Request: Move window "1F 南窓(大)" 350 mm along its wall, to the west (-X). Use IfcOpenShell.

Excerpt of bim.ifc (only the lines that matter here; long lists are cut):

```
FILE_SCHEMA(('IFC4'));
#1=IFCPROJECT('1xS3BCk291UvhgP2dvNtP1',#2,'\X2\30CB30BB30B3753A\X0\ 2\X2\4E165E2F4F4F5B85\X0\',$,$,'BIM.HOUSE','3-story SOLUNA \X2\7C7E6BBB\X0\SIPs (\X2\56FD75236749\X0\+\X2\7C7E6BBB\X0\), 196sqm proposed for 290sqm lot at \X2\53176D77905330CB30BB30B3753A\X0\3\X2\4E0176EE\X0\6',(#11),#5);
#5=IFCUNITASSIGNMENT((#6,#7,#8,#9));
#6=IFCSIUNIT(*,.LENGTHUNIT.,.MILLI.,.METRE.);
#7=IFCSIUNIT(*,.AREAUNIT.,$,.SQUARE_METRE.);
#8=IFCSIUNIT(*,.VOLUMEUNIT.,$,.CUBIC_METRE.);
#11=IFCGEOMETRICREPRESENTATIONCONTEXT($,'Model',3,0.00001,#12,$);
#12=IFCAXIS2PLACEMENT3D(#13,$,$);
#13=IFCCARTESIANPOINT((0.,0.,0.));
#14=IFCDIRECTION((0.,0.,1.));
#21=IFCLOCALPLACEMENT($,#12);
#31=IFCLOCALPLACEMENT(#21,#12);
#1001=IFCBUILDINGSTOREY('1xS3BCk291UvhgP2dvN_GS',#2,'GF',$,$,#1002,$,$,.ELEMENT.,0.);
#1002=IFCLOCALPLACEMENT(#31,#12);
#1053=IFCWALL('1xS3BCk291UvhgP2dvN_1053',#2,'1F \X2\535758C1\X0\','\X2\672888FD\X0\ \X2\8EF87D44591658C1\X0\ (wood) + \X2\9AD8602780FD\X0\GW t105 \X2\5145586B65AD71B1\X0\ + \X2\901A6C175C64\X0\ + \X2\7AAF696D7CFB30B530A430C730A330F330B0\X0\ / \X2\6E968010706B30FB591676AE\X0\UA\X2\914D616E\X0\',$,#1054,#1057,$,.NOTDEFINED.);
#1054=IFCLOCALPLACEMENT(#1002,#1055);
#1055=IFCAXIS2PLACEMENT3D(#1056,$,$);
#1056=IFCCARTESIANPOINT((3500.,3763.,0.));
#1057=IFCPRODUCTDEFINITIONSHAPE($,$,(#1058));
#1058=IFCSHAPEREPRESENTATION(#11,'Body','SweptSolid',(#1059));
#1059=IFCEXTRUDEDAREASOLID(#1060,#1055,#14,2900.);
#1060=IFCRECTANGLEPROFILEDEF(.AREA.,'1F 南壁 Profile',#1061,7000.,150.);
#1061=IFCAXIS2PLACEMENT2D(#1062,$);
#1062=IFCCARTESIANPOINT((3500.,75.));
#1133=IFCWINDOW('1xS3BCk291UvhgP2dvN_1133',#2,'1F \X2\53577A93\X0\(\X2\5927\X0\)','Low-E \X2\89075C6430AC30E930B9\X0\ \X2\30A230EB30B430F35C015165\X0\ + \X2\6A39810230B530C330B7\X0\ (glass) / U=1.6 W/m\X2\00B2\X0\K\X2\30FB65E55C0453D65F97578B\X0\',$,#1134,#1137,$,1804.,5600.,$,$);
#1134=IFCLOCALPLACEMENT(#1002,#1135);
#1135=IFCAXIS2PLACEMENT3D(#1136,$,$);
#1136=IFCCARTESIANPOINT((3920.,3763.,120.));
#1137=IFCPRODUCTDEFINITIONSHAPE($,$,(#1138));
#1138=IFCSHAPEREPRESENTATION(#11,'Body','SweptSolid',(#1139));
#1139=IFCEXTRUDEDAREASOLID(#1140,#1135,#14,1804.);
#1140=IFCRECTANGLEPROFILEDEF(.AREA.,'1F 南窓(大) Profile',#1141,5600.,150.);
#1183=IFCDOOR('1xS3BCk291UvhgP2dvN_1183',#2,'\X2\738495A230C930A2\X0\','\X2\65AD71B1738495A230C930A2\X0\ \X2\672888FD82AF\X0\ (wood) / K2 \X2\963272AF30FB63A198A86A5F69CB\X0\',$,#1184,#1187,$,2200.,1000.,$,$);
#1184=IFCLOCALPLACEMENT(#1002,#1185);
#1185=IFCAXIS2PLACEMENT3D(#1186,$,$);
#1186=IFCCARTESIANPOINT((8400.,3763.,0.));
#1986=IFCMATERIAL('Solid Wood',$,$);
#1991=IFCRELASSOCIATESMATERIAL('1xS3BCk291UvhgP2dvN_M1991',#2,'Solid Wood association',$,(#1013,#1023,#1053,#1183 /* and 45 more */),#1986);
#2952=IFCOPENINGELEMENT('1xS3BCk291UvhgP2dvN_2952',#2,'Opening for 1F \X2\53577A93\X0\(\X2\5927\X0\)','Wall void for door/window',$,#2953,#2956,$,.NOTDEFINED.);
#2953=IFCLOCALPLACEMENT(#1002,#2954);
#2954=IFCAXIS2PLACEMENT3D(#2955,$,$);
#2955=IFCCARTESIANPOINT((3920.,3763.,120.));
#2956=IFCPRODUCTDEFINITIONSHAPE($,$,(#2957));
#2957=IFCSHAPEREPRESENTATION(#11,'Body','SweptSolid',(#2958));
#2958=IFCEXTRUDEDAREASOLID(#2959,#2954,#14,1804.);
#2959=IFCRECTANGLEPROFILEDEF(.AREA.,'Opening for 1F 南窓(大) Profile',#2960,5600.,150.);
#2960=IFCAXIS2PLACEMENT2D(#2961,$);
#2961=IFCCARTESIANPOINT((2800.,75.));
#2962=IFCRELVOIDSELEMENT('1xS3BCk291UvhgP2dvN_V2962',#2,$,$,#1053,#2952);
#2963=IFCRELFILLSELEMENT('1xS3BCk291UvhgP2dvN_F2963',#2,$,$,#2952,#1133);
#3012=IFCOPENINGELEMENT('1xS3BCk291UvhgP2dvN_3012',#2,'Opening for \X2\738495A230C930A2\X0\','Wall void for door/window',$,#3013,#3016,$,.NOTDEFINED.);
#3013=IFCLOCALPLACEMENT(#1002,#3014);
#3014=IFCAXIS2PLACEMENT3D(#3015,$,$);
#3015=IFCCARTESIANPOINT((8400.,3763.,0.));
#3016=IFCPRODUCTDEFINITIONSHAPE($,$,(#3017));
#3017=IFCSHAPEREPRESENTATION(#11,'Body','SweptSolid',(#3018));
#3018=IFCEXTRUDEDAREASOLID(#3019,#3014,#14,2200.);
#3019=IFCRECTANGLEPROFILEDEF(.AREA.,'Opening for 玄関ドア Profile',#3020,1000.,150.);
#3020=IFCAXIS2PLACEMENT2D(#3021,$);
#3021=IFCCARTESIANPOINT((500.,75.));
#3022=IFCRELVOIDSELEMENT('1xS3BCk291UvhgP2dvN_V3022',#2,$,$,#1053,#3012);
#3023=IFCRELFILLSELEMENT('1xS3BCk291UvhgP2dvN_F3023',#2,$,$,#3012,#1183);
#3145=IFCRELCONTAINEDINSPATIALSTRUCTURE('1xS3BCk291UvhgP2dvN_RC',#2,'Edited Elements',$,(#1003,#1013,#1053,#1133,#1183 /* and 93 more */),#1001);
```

```python
import ifcopenshell
import ifcopenshell.api.geometry
import ifcopenshell.util.placement

model = ifcopenshell.open("bim.ifc")

window = model.by_id(1133)
opening = window.FillsVoids[0].RelatingOpeningElement
wall = opening.VoidsElements[0].RelatingBuildingElement

wall_matrix = ifcopenshell.util.placement.get_local_placement(wall.ObjectPlacement)
shift = wall_matrix[:3, 0] * -350.0
before = ifcopenshell.util.placement.get_local_placement(window.ObjectPlacement)[:3, 3].copy()

# The window is not placed relative to its opening, so move both.
for product in (opening, window):
    matrix = ifcopenshell.util.placement.get_local_placement(product.ObjectPlacement)
    matrix[:3, 3] += shift
    ifcopenshell.api.geometry.edit_object_placement(model, product=product, matrix=matrix, is_si=False)

after = ifcopenshell.util.placement.get_local_placement(window.ObjectPlacement)[:3, 3]
print("window moved by", (after - before).round(3) + 0.0)

model.write("bim_v2.ifc")
```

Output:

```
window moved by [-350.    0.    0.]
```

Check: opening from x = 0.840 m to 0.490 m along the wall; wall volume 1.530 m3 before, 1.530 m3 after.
